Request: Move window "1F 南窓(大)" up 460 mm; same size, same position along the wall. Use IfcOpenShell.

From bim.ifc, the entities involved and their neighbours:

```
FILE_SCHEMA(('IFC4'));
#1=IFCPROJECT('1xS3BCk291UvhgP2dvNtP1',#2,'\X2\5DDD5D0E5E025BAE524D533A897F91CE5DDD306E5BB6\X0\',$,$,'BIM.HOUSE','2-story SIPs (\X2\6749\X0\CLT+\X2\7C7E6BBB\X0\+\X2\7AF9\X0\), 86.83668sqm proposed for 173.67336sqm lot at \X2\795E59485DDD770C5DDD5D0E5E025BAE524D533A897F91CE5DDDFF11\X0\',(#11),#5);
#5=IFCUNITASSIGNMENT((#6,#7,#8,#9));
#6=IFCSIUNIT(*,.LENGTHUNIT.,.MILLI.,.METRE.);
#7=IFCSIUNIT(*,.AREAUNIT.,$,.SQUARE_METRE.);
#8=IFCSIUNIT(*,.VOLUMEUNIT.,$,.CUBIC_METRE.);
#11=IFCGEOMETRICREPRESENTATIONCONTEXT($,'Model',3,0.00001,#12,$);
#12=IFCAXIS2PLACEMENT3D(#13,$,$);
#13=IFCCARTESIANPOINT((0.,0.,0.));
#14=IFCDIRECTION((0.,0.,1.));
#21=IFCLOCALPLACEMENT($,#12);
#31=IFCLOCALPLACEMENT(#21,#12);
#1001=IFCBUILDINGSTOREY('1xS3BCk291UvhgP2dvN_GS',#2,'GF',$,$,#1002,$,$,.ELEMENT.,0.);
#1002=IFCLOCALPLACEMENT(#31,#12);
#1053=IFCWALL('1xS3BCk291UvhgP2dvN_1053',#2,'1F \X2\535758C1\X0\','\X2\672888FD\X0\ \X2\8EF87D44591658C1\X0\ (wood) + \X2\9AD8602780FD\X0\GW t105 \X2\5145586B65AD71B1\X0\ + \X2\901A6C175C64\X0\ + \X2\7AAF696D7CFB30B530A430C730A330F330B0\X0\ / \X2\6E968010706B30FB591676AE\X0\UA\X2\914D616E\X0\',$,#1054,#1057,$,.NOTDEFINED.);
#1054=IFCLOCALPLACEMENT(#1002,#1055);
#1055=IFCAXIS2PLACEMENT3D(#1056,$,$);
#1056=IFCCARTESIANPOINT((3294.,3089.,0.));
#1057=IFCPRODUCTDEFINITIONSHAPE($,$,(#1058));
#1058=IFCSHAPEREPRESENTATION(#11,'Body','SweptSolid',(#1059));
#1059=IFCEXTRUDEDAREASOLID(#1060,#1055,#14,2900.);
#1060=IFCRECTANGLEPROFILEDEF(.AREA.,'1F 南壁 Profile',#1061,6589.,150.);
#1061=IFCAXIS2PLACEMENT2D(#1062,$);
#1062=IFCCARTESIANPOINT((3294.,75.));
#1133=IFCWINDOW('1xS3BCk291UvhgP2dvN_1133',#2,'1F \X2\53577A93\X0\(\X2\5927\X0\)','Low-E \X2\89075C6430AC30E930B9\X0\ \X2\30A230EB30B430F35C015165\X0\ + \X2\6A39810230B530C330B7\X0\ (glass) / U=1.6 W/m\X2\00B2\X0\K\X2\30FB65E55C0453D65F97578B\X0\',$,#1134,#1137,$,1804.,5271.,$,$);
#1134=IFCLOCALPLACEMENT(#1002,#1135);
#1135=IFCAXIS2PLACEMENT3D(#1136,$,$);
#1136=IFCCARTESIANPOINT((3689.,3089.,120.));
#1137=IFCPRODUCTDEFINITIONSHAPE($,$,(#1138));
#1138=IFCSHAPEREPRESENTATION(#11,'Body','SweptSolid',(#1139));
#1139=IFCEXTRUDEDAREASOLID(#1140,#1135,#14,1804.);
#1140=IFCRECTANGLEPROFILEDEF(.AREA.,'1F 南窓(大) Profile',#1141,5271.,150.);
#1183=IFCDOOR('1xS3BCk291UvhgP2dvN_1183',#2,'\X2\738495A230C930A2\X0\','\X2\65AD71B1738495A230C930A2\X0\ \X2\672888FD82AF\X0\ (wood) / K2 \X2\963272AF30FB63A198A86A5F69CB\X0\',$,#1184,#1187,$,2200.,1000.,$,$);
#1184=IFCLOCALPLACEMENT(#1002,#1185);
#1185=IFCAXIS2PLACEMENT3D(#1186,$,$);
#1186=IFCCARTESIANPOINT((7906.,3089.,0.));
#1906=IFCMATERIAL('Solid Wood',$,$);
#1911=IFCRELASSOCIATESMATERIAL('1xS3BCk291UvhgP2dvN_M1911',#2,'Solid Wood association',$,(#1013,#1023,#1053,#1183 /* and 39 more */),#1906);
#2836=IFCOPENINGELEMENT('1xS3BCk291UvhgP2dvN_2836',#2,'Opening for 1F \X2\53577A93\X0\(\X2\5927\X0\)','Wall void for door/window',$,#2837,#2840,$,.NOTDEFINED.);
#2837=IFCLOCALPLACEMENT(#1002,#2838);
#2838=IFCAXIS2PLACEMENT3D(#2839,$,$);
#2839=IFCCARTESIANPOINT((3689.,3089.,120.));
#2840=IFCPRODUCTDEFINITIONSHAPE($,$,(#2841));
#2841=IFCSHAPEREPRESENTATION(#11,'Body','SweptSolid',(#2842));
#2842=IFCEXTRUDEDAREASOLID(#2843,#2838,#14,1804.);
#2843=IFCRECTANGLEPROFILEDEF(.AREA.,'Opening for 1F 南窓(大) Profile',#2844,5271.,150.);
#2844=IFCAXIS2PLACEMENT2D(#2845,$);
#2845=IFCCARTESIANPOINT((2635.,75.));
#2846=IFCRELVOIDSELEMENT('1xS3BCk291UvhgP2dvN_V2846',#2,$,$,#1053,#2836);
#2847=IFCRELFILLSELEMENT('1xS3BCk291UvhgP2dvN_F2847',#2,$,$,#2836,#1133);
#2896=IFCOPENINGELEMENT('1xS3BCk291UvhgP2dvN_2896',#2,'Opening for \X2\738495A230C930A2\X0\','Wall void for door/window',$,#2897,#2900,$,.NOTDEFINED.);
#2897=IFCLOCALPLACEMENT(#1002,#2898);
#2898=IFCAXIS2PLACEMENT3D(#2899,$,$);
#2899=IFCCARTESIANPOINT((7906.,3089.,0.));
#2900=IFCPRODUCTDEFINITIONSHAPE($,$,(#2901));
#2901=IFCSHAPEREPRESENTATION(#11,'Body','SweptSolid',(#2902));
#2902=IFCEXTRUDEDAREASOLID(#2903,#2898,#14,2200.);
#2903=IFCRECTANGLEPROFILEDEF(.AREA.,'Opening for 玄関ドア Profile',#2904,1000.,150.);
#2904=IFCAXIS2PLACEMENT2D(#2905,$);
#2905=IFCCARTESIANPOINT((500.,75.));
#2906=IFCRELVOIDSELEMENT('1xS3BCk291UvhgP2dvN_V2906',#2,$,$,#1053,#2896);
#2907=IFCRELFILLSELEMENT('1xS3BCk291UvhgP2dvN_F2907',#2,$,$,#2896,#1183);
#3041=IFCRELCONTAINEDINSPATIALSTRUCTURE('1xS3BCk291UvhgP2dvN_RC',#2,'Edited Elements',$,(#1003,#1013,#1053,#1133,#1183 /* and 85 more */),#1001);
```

```python
import numpy as np
import ifcopenshell
import ifcopenshell.api.geometry
import ifcopenshell.util.placement
import ifcopenshell.util.unit

model = ifcopenshell.open("bim.ifc")
unit_scale = ifcopenshell.util.unit.calculate_unit_scale(model)

window = model.by_id(1133)
opening = window.FillsVoids[0].RelatingOpeningElement
dz = 0.46 / unit_scale

shift = np.array([0.0, 0.0, dz])
# The window is not placed relative to its opening, so move both.
for product in (opening, window):
    matrix = ifcopenshell.util.placement.get_local_placement(product.ObjectPlacement)
    matrix[:3, 3] += shift
    ifcopenshell.api.geometry.edit_object_placement(model, product=product, matrix=matrix, is_si=False)

print(f"moved by {dz * unit_scale:+.3f} m")

model.write("bim_edited.ifc")
```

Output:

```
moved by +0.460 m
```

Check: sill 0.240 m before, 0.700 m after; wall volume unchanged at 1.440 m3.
